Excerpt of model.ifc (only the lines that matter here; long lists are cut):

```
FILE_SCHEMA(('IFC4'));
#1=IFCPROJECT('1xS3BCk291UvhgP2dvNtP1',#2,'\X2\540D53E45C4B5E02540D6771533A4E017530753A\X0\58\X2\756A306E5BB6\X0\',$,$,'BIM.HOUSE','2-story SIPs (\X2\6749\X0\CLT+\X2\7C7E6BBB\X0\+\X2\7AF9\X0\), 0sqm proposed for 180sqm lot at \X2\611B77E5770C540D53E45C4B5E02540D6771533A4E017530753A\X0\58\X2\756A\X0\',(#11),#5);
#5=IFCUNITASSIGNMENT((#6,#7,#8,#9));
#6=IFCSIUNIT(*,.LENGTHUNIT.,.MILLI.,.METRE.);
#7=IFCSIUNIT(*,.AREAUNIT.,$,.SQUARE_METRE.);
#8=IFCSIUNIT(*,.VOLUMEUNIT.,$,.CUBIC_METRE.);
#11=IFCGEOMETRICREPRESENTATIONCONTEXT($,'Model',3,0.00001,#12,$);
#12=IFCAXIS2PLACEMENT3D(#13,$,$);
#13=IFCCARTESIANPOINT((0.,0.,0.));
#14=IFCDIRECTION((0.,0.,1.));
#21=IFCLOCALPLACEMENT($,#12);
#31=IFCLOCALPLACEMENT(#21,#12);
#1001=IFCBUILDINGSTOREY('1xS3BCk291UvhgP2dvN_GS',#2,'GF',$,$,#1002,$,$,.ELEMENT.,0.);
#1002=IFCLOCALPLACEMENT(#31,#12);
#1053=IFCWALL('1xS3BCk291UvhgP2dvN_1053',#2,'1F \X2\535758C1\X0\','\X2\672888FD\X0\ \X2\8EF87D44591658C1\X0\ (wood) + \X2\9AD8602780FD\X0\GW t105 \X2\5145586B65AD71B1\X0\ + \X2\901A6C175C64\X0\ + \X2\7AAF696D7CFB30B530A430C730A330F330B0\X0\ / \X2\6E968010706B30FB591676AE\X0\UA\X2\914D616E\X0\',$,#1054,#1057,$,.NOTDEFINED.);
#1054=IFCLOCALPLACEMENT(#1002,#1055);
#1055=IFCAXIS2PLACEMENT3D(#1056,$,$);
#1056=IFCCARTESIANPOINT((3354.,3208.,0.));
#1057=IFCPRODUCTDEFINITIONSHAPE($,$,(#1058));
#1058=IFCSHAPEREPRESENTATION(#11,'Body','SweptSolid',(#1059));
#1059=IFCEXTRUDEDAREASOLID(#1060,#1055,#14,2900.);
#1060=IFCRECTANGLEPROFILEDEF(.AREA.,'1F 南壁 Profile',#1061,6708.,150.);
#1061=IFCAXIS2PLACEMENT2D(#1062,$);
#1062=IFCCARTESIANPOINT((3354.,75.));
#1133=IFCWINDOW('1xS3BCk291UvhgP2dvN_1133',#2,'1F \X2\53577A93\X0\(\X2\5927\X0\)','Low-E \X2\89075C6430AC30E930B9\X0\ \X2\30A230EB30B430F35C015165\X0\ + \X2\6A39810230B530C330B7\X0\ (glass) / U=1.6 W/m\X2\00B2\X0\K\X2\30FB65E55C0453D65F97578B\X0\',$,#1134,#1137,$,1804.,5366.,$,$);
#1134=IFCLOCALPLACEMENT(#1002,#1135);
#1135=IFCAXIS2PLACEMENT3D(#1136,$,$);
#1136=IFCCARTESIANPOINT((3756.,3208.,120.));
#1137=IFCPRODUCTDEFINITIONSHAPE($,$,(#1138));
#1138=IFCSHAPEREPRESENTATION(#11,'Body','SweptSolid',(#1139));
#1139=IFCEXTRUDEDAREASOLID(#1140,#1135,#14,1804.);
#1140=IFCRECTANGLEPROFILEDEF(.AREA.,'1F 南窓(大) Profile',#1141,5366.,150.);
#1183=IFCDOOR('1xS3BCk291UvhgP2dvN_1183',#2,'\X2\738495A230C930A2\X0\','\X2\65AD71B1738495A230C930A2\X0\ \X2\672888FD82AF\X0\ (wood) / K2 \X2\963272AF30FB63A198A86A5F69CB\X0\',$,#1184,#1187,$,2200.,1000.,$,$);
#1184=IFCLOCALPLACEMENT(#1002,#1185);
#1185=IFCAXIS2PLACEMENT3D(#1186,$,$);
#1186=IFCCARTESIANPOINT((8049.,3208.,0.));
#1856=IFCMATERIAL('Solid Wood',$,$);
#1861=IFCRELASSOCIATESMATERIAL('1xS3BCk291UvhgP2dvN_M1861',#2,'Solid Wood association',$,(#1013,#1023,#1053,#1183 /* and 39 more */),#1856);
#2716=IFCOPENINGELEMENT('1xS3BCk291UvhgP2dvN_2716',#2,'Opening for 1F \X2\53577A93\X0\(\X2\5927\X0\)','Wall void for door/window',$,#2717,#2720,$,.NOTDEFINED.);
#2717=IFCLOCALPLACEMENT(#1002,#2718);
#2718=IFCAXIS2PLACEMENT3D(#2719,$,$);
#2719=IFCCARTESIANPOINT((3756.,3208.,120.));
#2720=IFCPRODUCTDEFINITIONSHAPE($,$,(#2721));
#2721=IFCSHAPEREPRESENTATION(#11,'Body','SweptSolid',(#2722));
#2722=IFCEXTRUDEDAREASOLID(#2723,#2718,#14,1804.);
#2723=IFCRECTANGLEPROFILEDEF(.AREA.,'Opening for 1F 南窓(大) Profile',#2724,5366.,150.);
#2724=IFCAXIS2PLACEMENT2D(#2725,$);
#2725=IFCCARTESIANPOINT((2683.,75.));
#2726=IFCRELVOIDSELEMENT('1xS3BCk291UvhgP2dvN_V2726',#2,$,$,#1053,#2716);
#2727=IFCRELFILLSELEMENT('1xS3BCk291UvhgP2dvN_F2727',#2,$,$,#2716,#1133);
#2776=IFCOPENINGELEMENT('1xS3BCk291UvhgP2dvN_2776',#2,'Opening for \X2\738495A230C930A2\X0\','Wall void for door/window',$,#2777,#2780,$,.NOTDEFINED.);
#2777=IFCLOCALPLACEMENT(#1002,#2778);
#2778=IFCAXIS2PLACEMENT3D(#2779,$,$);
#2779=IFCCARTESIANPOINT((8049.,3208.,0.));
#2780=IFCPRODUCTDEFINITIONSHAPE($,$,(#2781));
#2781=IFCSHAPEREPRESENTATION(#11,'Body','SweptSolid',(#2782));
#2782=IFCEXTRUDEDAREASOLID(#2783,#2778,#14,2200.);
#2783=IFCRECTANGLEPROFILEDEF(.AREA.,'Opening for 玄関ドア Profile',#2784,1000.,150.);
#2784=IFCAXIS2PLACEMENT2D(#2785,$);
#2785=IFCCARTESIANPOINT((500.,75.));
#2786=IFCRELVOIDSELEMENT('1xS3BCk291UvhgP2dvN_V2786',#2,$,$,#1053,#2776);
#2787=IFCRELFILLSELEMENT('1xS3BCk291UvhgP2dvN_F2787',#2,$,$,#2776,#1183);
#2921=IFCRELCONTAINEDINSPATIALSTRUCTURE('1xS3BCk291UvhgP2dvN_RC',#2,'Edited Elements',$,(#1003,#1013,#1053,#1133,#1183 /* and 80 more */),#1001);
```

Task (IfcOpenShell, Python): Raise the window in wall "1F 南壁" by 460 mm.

```python
import numpy as np
import ifcopenshell
import ifcopenshell.api.geometry
import ifcopenshell.util.placement
import ifcopenshell.util.unit

model = ifcopenshell.open("model.ifc")
unit_scale = ifcopenshell.util.unit.calculate_unit_scale(model)

window = model.by_guid("1xS3BCk291UvhgP2dvN_1133")
opening = window.FillsVoids[0].RelatingOpeningElement
dz = 0.46 / unit_scale

shift = np.array([0.0, 0.0, dz])
# The window is not placed relative to its opening, so move both.
for product in (opening, window):
    matrix = ifcopenshell.util.placement.get_local_placement(product.ObjectPlacement)
    matrix[:3, 3] += shift
    ifcopenshell.api.geometry.edit_object_placement(model, product=product, matrix=matrix, is_si=False)

print(f"moved by {dz * unit_scale:+.3f} m")

model.write("model_edited.ifc")
```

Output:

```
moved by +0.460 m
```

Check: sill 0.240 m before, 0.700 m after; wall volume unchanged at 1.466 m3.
